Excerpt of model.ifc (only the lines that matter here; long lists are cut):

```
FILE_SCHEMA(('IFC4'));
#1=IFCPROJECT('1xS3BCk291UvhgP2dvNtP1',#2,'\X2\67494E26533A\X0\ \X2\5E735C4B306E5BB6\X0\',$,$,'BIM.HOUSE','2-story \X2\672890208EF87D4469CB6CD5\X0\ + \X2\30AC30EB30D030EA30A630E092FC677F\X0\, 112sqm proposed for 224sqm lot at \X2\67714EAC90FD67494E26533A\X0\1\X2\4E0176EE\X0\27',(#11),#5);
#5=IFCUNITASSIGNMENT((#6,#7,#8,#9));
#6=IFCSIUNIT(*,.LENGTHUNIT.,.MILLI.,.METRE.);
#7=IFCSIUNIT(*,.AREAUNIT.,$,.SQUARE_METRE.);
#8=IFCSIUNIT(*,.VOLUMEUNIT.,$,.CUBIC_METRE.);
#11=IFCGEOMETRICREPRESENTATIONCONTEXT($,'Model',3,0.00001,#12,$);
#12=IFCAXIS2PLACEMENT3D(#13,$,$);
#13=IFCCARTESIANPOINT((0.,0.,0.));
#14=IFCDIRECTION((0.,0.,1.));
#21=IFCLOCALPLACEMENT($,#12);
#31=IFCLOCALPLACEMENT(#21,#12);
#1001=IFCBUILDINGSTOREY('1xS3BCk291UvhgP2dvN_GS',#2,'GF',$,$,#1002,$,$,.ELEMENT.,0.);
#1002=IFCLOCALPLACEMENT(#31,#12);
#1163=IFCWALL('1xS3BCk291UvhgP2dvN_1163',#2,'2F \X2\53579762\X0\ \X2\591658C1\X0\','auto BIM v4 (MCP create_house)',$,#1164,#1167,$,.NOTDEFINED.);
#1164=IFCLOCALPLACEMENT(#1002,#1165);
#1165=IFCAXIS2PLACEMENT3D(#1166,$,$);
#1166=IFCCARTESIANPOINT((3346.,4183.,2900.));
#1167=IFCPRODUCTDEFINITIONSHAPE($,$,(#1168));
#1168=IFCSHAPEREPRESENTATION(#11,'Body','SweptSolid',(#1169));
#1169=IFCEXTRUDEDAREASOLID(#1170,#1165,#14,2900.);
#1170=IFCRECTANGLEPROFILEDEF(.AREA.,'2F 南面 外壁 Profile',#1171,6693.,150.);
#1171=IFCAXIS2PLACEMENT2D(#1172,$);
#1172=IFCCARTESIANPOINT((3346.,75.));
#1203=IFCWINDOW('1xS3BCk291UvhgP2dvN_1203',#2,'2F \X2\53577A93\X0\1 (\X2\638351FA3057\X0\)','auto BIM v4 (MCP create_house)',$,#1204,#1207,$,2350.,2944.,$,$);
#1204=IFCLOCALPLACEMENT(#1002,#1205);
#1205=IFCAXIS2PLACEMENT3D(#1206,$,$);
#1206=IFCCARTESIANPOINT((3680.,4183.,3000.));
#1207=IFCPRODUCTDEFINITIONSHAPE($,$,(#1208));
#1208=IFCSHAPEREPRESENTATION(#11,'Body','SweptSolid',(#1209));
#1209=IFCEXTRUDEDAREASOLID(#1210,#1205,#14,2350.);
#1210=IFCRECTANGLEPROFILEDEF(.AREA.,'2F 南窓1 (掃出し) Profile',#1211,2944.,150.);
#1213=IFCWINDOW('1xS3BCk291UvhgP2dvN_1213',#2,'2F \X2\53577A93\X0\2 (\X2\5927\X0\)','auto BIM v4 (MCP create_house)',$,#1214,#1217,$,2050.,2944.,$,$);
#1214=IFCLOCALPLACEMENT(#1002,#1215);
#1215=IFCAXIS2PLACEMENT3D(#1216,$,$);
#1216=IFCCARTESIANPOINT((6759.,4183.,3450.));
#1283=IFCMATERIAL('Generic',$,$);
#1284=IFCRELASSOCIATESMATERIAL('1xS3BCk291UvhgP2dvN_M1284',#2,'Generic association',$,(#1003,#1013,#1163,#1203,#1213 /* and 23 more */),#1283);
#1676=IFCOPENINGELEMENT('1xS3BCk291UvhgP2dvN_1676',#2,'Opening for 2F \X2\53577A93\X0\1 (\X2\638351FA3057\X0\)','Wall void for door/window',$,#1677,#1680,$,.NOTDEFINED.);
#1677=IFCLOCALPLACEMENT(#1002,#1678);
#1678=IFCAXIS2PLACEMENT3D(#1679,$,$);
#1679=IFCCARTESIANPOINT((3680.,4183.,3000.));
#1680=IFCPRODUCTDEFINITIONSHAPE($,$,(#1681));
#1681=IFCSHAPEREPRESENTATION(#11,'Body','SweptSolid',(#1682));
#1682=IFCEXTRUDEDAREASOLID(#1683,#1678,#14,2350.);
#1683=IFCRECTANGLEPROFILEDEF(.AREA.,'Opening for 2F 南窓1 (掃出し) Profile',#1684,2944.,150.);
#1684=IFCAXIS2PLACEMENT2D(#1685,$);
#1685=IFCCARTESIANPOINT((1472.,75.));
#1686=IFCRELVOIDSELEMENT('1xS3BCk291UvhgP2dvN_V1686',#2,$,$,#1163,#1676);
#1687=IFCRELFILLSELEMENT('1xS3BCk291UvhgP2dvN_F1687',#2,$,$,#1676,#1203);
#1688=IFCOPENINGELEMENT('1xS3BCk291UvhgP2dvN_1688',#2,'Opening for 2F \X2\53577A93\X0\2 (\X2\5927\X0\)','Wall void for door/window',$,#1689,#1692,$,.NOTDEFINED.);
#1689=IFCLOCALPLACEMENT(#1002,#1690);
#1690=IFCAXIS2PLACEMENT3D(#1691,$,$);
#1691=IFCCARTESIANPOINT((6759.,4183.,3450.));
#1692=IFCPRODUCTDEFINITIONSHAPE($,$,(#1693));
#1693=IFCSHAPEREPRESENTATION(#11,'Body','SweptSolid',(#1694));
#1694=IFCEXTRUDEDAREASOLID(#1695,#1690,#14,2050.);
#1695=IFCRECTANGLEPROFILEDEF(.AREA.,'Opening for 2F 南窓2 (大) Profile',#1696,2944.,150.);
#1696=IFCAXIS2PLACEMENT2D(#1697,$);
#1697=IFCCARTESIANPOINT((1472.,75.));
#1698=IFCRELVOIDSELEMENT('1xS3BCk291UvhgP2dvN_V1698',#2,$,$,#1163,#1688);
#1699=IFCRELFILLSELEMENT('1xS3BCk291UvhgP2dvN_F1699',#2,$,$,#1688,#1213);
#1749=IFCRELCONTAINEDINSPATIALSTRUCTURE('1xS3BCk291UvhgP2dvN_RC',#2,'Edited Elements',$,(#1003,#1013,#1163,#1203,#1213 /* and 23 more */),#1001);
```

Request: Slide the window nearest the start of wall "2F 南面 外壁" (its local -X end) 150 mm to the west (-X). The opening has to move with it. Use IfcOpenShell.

```python
import ifcopenshell
import ifcopenshell.api.geometry
import ifcopenshell.util.placement

model = ifcopenshell.open("model.ifc")

window = model.by_id(1203)
opening = window.FillsVoids[0].RelatingOpeningElement
wall = opening.VoidsElements[0].RelatingBuildingElement

wall_matrix = ifcopenshell.util.placement.get_local_placement(wall.ObjectPlacement)
shift = wall_matrix[:3, 0] * -150.0
before = ifcopenshell.util.placement.get_local_placement(window.ObjectPlacement)[:3, 3].copy()

# The window is not placed relative to its opening, so move both.
for product in (opening, window):
    matrix = ifcopenshell.util.placement.get_local_placement(product.ObjectPlacement)
    matrix[:3, 3] += shift
    ifcopenshell.api.geometry.edit_object_placement(model, product=product, matrix=matrix, is_si=False)

after = ifcopenshell.util.placement.get_local_placement(window.ObjectPlacement)[:3, 3]
print("window moved by", (after - before).round(3) + 0.0)

model.write("model_v2.ifc")
```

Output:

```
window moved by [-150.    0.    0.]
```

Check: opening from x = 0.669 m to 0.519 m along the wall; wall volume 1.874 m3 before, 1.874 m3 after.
